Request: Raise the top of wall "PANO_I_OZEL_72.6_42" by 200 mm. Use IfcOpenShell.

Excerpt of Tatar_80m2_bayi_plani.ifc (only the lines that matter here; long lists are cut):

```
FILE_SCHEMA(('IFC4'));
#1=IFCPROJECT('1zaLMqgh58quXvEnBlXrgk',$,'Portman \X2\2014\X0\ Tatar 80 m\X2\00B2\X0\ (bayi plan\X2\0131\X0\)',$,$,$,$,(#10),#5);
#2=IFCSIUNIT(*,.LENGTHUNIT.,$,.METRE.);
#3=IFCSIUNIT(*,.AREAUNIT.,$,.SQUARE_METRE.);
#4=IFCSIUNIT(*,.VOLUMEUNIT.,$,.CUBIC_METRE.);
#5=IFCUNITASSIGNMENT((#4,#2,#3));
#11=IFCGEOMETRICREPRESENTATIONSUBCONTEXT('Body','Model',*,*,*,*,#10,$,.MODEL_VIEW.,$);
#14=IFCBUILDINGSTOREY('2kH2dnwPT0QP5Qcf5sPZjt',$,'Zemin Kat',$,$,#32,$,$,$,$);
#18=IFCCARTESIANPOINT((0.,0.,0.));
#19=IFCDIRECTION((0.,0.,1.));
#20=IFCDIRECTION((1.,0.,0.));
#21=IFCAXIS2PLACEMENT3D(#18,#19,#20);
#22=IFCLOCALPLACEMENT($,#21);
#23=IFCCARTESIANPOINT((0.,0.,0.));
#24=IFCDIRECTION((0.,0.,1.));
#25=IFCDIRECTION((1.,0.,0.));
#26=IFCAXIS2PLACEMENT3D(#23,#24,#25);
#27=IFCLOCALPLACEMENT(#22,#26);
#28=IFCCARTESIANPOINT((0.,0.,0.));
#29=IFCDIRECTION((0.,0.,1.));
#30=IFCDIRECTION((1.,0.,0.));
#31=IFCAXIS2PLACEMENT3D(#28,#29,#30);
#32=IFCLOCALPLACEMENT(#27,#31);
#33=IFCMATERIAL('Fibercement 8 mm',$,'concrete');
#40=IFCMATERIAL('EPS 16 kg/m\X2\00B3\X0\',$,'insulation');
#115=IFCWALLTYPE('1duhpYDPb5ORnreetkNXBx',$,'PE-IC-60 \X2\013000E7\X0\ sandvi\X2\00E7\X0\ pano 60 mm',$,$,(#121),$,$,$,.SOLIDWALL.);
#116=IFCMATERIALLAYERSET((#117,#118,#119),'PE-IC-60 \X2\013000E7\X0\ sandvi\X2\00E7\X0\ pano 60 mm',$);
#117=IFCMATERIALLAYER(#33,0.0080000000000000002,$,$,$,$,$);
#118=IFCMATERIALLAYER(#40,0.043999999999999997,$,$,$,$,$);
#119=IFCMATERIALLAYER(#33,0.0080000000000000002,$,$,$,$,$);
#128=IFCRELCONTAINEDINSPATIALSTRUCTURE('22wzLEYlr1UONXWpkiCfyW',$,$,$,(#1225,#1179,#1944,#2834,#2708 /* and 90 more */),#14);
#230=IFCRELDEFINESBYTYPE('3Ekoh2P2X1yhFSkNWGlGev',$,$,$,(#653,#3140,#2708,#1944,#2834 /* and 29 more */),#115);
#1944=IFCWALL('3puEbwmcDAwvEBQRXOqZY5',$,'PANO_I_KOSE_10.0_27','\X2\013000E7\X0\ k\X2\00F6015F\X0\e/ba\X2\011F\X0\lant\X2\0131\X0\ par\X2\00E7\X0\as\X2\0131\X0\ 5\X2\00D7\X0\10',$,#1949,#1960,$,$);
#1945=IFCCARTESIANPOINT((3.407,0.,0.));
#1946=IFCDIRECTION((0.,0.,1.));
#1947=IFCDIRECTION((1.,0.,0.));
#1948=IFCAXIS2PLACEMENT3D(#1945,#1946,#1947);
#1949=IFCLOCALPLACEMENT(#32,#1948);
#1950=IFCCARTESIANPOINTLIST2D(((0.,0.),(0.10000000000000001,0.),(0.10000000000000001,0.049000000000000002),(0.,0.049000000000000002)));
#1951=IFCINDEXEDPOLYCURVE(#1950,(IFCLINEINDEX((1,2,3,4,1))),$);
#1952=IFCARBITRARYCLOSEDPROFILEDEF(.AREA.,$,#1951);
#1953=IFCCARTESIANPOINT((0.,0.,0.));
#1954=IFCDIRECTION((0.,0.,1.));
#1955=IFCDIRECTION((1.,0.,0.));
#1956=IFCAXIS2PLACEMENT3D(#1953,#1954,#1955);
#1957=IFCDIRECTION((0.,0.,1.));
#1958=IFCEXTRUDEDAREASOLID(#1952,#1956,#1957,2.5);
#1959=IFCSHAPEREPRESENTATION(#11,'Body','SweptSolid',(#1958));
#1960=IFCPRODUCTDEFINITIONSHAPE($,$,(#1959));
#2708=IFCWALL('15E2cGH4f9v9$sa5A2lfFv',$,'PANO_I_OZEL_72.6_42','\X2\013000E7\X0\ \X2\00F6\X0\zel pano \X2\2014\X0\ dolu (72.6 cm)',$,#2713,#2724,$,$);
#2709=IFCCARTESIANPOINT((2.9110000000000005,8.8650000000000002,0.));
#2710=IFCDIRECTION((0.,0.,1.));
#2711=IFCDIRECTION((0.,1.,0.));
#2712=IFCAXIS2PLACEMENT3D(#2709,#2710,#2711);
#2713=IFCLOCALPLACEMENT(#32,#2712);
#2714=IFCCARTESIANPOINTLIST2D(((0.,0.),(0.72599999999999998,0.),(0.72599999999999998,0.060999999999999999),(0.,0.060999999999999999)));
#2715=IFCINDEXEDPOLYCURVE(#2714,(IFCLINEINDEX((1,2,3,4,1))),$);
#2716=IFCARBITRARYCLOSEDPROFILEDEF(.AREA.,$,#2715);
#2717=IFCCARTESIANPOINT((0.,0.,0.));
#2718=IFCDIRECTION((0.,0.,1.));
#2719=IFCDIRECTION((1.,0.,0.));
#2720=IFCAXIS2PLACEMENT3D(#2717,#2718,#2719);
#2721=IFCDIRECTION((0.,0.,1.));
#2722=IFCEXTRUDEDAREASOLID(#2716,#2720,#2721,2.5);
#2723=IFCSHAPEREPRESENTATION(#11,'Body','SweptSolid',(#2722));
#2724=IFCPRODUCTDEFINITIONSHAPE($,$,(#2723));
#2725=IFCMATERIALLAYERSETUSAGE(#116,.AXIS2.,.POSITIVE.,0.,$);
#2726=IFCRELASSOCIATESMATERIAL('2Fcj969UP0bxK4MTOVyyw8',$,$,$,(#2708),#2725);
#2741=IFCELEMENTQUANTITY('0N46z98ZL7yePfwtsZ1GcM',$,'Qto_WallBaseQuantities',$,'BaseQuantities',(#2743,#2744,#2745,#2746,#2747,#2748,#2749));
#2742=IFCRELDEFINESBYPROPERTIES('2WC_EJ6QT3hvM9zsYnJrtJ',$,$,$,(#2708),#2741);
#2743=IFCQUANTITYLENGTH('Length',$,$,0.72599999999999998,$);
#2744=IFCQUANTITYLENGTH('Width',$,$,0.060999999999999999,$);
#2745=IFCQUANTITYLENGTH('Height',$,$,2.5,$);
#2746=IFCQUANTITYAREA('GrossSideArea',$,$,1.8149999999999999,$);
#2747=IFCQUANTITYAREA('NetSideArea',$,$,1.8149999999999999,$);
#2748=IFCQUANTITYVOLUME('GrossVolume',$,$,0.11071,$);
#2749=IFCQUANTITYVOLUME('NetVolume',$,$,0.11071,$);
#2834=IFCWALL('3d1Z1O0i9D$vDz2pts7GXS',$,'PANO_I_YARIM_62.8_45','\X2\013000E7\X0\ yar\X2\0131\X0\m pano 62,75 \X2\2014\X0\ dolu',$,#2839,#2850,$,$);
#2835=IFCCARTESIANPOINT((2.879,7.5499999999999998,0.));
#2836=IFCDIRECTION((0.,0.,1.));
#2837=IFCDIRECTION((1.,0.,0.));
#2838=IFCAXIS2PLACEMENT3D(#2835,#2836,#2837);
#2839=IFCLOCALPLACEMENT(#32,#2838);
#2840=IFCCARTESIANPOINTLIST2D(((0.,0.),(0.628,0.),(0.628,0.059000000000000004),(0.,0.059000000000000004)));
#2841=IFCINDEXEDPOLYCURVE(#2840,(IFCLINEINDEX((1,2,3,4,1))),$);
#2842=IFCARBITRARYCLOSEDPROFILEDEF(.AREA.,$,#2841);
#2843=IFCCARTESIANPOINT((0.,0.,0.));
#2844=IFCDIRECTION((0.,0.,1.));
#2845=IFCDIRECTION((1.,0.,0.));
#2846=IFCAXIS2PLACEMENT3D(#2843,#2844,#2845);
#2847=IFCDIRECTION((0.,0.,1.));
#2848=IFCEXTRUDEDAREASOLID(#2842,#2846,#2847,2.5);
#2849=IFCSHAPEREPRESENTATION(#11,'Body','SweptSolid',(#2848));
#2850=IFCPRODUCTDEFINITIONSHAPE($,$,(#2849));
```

```python
import ifcopenshell
import ifcopenshell.api.pset
import ifcopenshell.geom
import ifcopenshell.util.element
import ifcopenshell.util.representation
import ifcopenshell.util.shape
import ifcopenshell.util.unit

model = ifcopenshell.open("Tatar_80m2_bayi_plani.ifc")
unit_scale = ifcopenshell.util.unit.calculate_unit_scale(model)
area_scale = ifcopenshell.util.unit.calculate_unit_scale(model, "AREAUNIT")
volume_scale = ifcopenshell.util.unit.calculate_unit_scale(model, "VOLUMEUNIT")
settings = ifcopenshell.geom.settings()


def volume(element):
    """Net volume in cubic metres, openings subtracted."""
    shape = ifcopenshell.geom.create_shape(settings, element)
    return ifcopenshell.util.shape.get_volume(shape.geometry)


wall = model.by_guid("15E2cGH4f9v9$sa5A2lfFv")
before = volume(wall)

body = ifcopenshell.util.representation.get_representation(wall, "Model", "Body")
solid = body.Items[0]
old_height = solid.Depth
solid.Depth += 0.2 / unit_scale
after = volume(wall)
thickness = 0.061  # wall thickness in metres

# Update the stored height, areas and volumes.
qto = model.by_id(ifcopenshell.util.element.get_pset(wall, "Qto_WallBaseQuantities", should_inherit=False)["id"])
ifcopenshell.api.pset.edit_qto(model, qto=qto, properties={
    "Height": solid.Depth,
    "GrossSideArea": ifcopenshell.util.element.get_pset(wall, "Qto_WallBaseQuantities", "GrossSideArea") * solid.Depth / old_height,
    "NetSideArea": after / thickness / area_scale,
    "GrossVolume": ifcopenshell.util.element.get_pset(wall, "Qto_WallBaseQuantities", "GrossVolume") * solid.Depth / old_height,
    "NetVolume": after / volume_scale,
})

print(f"height {old_height:g} -> {solid.Depth:g}, volume {before:.3f} -> {after:.3f} m3")

model.write("Tatar_80m2_bayi_plani_edited.ifc")
```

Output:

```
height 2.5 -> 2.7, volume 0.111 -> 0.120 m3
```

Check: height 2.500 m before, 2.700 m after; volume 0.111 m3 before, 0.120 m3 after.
